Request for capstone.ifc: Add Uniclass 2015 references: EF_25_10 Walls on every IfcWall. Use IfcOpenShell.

First a look at what the model holds.

```python
import ifcopenshell

model = ifcopenshell.open("capstone.ifc")
print(model.schema)
print("classifications:", [c.Name for c in model.by_type("IfcClassification")])
for ifc_class in ("IfcDoor", "IfcRoof", "IfcStair", "IfcWall", "IfcWindow"):
    print(ifc_class, len(model.by_type(ifc_class)))
```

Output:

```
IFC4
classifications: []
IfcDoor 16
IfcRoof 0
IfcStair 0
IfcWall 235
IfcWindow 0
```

```python
import ifcopenshell
import ifcopenshell.api.classification

model = ifcopenshell.open("capstone.ifc")

system = ifcopenshell.api.classification.add_classification(model, classification="Uniclass 2015")

codes = {
    "IfcWall": ("EF_25_10", "Walls"),
}
for ifc_class, (code, name) in codes.items():
    products = model.by_type(ifc_class)
    ifcopenshell.api.classification.add_reference(
        model, products=products, classification=system, identification=code, name=name
    )
    print(code, len(products))

model.write("capstone_rev.ifc")
```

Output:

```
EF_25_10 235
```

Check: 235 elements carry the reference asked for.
